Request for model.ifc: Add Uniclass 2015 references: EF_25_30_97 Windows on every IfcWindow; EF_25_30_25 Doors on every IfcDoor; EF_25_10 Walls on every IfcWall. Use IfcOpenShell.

First a look at what the model holds.

```python
import ifcopenshell

model = ifcopenshell.open("model.ifc")
print(model.schema)
print("classifications:", [c.Name for c in model.by_type("IfcClassification")])
for ifc_class in ("IfcDoor", "IfcRoof", "IfcStair", "IfcWall", "IfcWindow"):
    print(ifc_class, len(model.by_type(ifc_class)))
```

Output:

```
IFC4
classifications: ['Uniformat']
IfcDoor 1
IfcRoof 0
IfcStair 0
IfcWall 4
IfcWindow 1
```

```python
import ifcopenshell
import ifcopenshell.api.classification

model = ifcopenshell.open("model.ifc")

system = ifcopenshell.api.classification.add_classification(model, classification="Uniclass 2015")

codes = {
    "IfcWindow": ("EF_25_30_97", "Windows"),
    "IfcDoor": ("EF_25_30_25", "Doors"),
    "IfcWall": ("EF_25_10", "Walls"),
}
for ifc_class, (code, name) in codes.items():
    products = model.by_type(ifc_class)
    ifcopenshell.api.classification.add_reference(
        model, products=products, classification=system, identification=code, name=name
    )
    print(code, len(products))

model.write("model_rev.ifc")
```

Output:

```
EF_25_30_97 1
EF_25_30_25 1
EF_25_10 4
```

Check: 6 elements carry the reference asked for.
